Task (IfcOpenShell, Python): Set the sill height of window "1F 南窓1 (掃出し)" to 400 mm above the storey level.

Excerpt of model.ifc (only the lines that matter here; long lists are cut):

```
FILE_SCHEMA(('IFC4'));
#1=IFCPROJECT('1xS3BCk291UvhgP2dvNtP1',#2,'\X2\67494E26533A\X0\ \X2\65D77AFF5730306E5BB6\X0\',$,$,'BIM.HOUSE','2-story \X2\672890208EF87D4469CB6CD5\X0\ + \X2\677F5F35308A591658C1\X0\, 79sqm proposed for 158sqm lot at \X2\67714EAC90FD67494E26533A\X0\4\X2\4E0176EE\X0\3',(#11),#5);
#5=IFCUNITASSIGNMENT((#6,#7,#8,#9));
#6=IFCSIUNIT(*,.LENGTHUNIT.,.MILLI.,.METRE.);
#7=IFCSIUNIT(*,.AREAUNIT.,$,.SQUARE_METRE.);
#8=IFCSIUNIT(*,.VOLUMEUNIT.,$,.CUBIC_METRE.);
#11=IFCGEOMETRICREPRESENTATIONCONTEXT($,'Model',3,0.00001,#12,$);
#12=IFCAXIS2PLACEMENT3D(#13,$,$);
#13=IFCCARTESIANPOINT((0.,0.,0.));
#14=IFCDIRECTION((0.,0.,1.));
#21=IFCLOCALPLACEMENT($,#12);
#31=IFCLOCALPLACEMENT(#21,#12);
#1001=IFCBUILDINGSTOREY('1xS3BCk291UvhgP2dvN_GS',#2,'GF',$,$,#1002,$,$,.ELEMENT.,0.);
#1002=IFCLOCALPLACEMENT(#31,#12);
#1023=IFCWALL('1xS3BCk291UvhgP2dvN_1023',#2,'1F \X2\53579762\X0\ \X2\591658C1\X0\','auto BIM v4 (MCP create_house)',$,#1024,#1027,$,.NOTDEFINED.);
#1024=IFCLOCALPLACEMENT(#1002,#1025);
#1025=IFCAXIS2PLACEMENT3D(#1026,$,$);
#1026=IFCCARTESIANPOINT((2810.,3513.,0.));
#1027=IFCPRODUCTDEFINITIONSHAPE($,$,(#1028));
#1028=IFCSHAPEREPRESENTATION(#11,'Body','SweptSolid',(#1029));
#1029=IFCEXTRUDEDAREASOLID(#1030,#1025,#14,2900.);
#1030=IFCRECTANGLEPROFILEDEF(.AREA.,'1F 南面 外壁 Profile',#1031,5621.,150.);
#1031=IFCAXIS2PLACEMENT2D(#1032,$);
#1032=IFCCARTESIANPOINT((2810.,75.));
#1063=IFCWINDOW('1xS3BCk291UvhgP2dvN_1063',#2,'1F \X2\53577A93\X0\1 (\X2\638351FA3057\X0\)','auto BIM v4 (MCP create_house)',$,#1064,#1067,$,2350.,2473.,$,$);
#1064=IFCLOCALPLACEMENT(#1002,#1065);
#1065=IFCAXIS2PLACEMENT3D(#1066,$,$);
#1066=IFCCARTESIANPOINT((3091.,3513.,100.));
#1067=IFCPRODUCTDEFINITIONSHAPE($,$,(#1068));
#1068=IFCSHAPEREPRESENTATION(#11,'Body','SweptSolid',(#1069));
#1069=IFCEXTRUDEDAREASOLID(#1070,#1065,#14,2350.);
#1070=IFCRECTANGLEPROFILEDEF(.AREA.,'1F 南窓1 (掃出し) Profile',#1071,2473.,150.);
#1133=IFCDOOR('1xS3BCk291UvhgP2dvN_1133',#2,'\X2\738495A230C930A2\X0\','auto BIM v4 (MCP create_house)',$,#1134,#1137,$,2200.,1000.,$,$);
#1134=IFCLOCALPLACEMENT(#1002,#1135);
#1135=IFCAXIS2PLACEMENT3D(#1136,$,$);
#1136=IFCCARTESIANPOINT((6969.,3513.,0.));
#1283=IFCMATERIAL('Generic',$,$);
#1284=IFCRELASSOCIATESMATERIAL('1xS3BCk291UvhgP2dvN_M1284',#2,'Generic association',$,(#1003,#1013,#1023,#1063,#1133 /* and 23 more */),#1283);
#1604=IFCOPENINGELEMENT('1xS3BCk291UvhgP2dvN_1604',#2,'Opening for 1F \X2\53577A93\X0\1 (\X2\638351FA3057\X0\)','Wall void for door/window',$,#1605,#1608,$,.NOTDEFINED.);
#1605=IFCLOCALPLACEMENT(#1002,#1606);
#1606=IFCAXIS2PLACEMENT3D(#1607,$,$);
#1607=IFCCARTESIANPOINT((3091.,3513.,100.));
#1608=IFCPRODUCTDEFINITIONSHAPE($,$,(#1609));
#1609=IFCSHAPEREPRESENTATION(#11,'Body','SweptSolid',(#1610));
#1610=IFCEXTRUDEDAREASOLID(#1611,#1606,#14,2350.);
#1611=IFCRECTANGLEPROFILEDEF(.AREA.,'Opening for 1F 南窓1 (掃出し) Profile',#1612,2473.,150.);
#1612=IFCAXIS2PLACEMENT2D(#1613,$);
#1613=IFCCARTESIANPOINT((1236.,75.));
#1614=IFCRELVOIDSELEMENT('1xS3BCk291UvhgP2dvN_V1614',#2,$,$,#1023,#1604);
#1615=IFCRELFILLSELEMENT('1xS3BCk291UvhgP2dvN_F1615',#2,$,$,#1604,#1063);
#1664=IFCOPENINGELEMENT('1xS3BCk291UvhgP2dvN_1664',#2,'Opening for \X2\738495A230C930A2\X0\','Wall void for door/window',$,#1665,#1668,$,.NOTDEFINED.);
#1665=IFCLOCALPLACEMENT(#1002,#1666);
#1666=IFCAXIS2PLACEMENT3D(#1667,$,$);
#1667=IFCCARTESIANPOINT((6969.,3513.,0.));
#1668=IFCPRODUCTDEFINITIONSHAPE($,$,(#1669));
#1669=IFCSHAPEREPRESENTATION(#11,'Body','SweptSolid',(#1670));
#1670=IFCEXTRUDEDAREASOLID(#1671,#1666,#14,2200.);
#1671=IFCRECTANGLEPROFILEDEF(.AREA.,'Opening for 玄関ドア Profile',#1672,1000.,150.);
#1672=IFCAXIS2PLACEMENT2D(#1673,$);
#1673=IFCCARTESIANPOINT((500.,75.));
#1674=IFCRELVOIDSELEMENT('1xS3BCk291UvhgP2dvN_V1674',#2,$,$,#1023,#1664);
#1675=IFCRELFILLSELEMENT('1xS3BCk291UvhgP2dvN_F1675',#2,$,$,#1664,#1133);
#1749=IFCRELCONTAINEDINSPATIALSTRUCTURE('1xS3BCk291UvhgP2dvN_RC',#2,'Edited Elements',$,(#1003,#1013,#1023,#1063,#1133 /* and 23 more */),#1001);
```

```python
import numpy as np
import ifcopenshell
import ifcopenshell.api.geometry
import ifcopenshell.geom
import ifcopenshell.util.element
import ifcopenshell.util.placement
import ifcopenshell.util.shape
import ifcopenshell.util.unit

model = ifcopenshell.open("model.ifc")
unit_scale = ifcopenshell.util.unit.calculate_unit_scale(model)

window = model.by_guid("1xS3BCk291UvhgP2dvN_1063")
opening = window.FillsVoids[0].RelatingOpeningElement
storey = ifcopenshell.util.element.get_container(window, ifc_class="IfcBuildingStorey")
level = ifcopenshell.util.placement.get_local_placement(storey.ObjectPlacement)[2, 3]

# The opening's origin need not be at the sill, so measure its lowest point.
shape = ifcopenshell.geom.create_shape(ifcopenshell.geom.settings(), opening)
bottom = ifcopenshell.util.shape.get_shape_bottom_elevation(shape, shape.geometry) / unit_scale
dz = level + 0.4 / unit_scale - bottom

shift = np.array([0.0, 0.0, dz])
# The window is not placed relative to its opening, so move both.
for product in (opening, window):
    matrix = ifcopenshell.util.placement.get_local_placement(product.ObjectPlacement)
    matrix[:3, 3] += shift
    ifcopenshell.api.geometry.edit_object_placement(model, product=product, matrix=matrix, is_si=False)

print(f"moved by {dz * unit_scale:+.3f} m")

model.write("model_edited.ifc")
```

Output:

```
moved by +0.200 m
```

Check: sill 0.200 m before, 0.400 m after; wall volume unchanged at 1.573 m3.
